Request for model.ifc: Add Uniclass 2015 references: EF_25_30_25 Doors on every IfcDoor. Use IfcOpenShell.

First a look at what the model holds.

```python
import ifcopenshell

model = ifcopenshell.open("model.ifc")
print(model.schema)
print("classifications:", [c.Name for c in model.by_type("IfcClassification")])
for ifc_class in ("IfcDoor", "IfcRoof", "IfcStair", "IfcWall", "IfcWindow"):
    print(ifc_class, len(model.by_type(ifc_class)))
```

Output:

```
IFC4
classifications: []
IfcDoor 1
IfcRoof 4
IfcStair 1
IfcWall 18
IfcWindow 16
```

```python
import ifcopenshell
import ifcopenshell.api.classification

model = ifcopenshell.open("model.ifc")

system = ifcopenshell.api.classification.add_classification(model, classification="Uniclass 2015")

codes = {
    "IfcDoor": ("EF_25_30_25", "Doors"),
}
for ifc_class, (code, name) in codes.items():
    products = model.by_type(ifc_class)
    ifcopenshell.api.classification.add_reference(
        model, products=products, classification=system, identification=code, name=name
    )
    print(code, len(products))

model.write("model_updated.ifc")
```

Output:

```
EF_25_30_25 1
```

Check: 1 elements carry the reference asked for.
